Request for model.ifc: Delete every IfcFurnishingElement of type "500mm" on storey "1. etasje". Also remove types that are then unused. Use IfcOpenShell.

First a look at what the model holds.

```python
import ifcopenshell
import ifcopenshell.util.element

model = ifcopenshell.open("model.ifc")
print(model.schema)
storey = next(s for s in model.by_type("IfcBuildingStorey") if s.Name == "1. etasje")
furniture = [e for e in ifcopenshell.util.element.get_decomposition(storey) if e.is_a("IfcFurnishingElement")]
seen = {}
for e in furniture:
    element_type = ifcopenshell.util.element.get_type(e)
    name = element_type.Name if element_type not in (None, e) else None
    seen[name] = seen.get(name, 0) + 1
for name, count in sorted(seen.items(), key=str):
    print(count, "x", name)
```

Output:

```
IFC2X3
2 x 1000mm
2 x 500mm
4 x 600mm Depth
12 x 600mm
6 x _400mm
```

```python
import ifcopenshell
import ifcopenshell.api.root
import ifcopenshell.util.element

model = ifcopenshell.open("model.ifc")

storey = next(s for s in model.by_type("IfcBuildingStorey") if s.Name == "1. etasje")
furniture = [e for e in ifcopenshell.util.element.get_decomposition(storey) if e.is_a("IfcFurnishingElement")]
targets = [e for e in furniture if (t := ifcopenshell.util.element.get_type(e)) not in (None, e) and t.Name == "500mm"]
types = {ifcopenshell.util.element.get_type(e) for e in targets} - {None, *targets}

for e in targets:
    ifcopenshell.api.root.remove_product(model, product=e)
print(len(targets), "removed")

unused = [t for t in types if not ifcopenshell.util.element.get_types(t)]
for t in unused:
    ifcopenshell.api.root.remove_product(model, product=t)
print(len(unused), "unused types removed")

model.write("model_edited.ifc")
```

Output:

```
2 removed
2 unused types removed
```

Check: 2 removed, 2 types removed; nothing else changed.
